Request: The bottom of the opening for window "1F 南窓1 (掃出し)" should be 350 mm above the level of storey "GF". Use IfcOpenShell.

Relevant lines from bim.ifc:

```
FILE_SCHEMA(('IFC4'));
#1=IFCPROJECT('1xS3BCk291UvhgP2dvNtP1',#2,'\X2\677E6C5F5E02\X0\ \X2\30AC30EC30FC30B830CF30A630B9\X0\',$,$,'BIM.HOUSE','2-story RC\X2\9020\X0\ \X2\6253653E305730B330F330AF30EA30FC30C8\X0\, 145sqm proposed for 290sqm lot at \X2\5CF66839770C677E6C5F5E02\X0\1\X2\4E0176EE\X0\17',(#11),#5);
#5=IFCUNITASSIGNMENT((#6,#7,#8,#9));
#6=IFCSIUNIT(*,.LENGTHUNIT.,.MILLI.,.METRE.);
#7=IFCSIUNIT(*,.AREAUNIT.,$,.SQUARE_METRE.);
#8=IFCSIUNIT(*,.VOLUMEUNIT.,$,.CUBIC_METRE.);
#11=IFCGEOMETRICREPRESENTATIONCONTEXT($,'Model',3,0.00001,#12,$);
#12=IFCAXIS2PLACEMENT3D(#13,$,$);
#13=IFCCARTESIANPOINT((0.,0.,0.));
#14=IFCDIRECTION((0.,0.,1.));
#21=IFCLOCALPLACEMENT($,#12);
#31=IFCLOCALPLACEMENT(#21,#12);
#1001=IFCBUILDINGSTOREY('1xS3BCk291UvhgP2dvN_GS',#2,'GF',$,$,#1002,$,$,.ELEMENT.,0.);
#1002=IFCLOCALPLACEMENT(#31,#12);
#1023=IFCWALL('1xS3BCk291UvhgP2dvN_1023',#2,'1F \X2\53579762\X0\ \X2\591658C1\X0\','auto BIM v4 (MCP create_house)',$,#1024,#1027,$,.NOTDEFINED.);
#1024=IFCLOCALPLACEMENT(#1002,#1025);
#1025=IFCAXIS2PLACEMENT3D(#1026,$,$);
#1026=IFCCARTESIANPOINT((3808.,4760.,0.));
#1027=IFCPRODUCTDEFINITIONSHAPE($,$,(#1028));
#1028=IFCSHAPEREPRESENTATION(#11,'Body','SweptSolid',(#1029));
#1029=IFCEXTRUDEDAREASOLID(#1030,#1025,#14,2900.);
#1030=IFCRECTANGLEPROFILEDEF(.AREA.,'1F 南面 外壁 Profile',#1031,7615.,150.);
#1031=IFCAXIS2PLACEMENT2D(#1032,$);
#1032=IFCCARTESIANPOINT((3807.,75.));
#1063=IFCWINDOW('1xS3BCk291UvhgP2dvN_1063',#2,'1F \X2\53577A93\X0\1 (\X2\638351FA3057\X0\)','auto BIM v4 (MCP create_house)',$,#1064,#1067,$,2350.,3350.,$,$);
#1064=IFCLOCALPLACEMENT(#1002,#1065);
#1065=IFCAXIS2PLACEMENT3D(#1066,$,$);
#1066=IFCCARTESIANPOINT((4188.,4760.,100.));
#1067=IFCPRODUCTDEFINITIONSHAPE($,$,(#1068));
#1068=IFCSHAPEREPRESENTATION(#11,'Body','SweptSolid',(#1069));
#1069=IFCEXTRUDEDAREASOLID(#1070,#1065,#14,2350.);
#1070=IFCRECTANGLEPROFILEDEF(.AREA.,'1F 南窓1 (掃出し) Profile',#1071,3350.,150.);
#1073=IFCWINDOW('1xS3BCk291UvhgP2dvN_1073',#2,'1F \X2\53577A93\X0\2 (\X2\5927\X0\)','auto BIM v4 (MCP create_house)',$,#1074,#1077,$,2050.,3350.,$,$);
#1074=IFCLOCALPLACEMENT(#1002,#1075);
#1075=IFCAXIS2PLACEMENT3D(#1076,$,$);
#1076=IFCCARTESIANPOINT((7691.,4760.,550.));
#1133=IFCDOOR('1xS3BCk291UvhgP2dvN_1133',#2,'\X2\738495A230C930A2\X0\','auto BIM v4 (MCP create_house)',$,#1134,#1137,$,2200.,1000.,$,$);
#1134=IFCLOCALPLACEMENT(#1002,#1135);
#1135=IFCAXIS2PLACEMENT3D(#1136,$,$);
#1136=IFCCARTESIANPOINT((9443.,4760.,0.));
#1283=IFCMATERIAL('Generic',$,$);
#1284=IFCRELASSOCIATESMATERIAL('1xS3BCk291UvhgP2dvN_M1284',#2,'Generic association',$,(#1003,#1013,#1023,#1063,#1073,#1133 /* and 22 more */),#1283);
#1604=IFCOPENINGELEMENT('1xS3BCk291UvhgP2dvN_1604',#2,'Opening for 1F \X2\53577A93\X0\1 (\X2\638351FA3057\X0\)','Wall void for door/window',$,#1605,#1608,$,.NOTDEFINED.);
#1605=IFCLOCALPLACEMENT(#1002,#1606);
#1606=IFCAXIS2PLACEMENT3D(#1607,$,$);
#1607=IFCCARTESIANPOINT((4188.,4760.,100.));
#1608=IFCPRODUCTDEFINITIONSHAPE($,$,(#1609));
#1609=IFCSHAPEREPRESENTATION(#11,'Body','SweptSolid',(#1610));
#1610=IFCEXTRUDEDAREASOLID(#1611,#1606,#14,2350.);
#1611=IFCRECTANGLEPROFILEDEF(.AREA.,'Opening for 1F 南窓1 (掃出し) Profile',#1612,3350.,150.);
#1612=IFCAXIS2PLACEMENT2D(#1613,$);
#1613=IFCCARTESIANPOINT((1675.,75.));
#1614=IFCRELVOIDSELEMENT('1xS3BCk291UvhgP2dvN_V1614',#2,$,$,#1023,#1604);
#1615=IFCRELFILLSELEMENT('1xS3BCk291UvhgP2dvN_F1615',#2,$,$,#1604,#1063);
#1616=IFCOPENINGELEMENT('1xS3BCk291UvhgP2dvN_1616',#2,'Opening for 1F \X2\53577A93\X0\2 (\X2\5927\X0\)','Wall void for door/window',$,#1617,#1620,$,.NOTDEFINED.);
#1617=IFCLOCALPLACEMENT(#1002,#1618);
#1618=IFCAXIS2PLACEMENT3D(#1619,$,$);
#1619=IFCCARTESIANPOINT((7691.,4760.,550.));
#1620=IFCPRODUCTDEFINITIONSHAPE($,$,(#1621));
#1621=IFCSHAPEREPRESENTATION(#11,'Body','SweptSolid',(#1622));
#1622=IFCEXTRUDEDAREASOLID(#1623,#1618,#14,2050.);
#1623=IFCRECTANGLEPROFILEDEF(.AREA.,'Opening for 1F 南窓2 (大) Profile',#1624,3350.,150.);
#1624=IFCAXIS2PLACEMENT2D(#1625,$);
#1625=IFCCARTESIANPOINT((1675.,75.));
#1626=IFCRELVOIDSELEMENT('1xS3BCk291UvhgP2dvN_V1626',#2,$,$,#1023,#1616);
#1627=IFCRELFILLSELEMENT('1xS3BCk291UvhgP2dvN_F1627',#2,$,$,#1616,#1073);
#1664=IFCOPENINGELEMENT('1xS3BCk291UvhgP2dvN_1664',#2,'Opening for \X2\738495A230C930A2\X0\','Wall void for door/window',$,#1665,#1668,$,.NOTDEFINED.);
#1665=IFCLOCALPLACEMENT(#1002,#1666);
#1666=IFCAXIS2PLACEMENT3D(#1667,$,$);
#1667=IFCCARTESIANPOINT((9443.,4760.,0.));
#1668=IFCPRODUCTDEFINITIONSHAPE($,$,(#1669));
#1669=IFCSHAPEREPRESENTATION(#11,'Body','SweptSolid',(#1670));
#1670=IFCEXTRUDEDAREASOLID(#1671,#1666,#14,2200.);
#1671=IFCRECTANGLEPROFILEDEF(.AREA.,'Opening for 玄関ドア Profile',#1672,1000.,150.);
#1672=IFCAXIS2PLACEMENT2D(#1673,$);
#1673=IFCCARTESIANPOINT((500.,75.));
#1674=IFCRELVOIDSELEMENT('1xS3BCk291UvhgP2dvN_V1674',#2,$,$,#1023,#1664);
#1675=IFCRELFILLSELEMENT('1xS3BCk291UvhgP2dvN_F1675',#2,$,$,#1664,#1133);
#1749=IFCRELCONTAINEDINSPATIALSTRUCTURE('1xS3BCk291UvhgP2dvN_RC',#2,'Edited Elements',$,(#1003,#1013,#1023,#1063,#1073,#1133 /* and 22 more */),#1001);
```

```python
import numpy as np
import ifcopenshell
import ifcopenshell.api.geometry
import ifcopenshell.geom
import ifcopenshell.util.element
import ifcopenshell.util.placement
import ifcopenshell.util.shape
import ifcopenshell.util.unit

model = ifcopenshell.open("bim.ifc")
unit_scale = ifcopenshell.util.unit.calculate_unit_scale(model)

window = model.by_guid("1xS3BCk291UvhgP2dvN_1063")
opening = window.FillsVoids[0].RelatingOpeningElement
storey = ifcopenshell.util.element.get_container(window, ifc_class="IfcBuildingStorey")
level = ifcopenshell.util.placement.get_local_placement(storey.ObjectPlacement)[2, 3]

# The opening's origin need not be at the sill, so measure its lowest point.
shape = ifcopenshell.geom.create_shape(ifcopenshell.geom.settings(), opening)
bottom = ifcopenshell.util.shape.get_shape_bottom_elevation(shape, shape.geometry) / unit_scale
dz = level + 0.35 / unit_scale - bottom

shift = np.array([0.0, 0.0, dz])
# The window is not placed relative to its opening, so move both.
for product in (opening, window):
    matrix = ifcopenshell.util.placement.get_local_placement(product.ObjectPlacement)
    matrix[:3, 3] += shift
    ifcopenshell.api.geometry.edit_object_placement(model, product=product, matrix=matrix, is_si=False)

print(f"moved by {dz * unit_scale:+.3f} m")

model.write("bim_edited.ifc")
```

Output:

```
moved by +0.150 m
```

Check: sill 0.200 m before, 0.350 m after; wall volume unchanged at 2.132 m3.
